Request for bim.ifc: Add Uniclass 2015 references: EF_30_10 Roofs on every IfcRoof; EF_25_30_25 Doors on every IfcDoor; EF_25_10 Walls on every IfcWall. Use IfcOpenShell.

First a look at what the model holds.

```python
import ifcopenshell

model = ifcopenshell.open("bim.ifc")
print(model.schema)
print("classifications:", [c.Name for c in model.by_type("IfcClassification")])
for ifc_class in ("IfcDoor", "IfcRoof", "IfcStair", "IfcWall", "IfcWindow"):
    print(ifc_class, len(model.by_type(ifc_class)))
```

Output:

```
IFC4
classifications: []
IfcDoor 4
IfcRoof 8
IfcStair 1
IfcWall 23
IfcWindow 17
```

```python
import ifcopenshell
import ifcopenshell.api.classification

model = ifcopenshell.open("bim.ifc")

system = ifcopenshell.api.classification.add_classification(model, classification="Uniclass 2015")

codes = {
    "IfcRoof": ("EF_30_10", "Roofs"),
    "IfcDoor": ("EF_25_30_25", "Doors"),
    "IfcWall": ("EF_25_10", "Walls"),
}
for ifc_class, (code, name) in codes.items():
    products = model.by_type(ifc_class)
    ifcopenshell.api.classification.add_reference(
        model, products=products, classification=system, identification=code, name=name
    )
    print(code, len(products))

model.write("bim-out.ifc")
```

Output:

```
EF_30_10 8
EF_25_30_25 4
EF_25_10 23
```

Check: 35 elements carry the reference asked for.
